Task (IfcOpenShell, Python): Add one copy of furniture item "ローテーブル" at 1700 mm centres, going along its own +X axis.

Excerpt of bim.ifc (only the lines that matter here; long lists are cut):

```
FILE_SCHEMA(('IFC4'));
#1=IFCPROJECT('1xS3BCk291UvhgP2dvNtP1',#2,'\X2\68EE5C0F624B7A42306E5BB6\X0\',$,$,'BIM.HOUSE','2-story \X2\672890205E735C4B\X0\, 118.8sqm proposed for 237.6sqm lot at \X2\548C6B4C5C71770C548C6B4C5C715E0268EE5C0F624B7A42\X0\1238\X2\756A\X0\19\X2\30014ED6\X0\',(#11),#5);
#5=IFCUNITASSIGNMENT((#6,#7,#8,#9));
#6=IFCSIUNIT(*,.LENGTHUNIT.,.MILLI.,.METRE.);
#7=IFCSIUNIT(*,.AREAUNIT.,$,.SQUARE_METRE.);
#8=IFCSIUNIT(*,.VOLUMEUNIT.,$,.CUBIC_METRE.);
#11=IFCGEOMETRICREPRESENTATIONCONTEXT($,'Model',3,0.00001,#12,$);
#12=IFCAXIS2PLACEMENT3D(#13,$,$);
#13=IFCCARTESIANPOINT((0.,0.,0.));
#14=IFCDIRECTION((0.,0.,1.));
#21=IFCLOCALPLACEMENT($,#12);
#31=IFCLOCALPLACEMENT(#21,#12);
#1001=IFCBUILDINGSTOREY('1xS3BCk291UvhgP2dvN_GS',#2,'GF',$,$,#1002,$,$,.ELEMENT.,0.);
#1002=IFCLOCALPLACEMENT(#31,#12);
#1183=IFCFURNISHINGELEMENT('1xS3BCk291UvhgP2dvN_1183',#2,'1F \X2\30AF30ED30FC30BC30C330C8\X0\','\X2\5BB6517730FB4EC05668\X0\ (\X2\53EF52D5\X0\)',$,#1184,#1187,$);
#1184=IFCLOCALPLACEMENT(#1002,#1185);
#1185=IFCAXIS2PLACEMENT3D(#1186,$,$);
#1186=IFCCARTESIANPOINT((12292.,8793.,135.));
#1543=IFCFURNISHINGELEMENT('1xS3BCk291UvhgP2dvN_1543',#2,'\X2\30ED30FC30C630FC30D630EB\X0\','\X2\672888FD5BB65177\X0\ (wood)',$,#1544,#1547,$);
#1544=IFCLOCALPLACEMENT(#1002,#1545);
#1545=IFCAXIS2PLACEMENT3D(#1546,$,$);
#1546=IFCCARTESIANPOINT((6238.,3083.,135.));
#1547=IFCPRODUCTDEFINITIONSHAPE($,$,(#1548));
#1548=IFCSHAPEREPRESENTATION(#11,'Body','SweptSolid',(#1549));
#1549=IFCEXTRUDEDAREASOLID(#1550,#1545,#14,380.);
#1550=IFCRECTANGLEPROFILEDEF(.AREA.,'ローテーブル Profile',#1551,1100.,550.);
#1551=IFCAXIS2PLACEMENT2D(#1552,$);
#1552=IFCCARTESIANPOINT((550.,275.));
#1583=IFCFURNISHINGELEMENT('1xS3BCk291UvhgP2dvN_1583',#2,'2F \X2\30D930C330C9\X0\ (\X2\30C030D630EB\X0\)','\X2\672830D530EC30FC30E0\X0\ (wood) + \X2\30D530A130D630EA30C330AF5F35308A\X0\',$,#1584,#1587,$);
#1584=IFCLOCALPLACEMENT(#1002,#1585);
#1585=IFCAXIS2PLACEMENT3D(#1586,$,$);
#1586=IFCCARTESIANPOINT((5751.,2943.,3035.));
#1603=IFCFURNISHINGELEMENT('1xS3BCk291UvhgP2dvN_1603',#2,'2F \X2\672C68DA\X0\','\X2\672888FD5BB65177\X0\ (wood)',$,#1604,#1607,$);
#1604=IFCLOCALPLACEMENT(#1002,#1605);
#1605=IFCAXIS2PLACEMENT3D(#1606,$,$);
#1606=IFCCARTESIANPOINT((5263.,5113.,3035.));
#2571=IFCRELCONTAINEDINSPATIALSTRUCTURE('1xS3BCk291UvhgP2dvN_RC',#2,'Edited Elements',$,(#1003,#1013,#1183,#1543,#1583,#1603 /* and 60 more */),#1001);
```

```python
import ifcopenshell
import ifcopenshell.api.geometry
import ifcopenshell.api.root
import ifcopenshell.util.element
import ifcopenshell.util.placement
import ifcopenshell.util.unit

model = ifcopenshell.open("bim.ifc")
unit_scale = ifcopenshell.util.unit.calculate_unit_scale(model)


def reuse_history(source, copy):
    """copy_class also copies each property set's owner history, people and application; keep the originals."""
    for rel in copy.IsDefinedBy:
        if rel.is_a("IfcRelDefinesByProperties") and (history := rel.RelatingPropertyDefinition.OwnerHistory):
            rel.RelatingPropertyDefinition.OwnerHistory = source.OwnerHistory
            ifcopenshell.util.element.remove_deep2(model, history)


source = model.by_guid("1xS3BCk291UvhgP2dvN_1543")
base = ifcopenshell.util.placement.get_local_placement(source.ObjectPlacement)
step = base[:3, 0] * 1.7 / unit_scale

for i in range(1, 2):
    copy = ifcopenshell.api.root.copy_class(model, product=source)
    copy.Representation = ifcopenshell.util.element.copy_deep(
        model, source.Representation, exclude=["IfcGeometricRepresentationContext", "IfcRepresentationMap"]
    )
    reuse_history(source, copy)
    matrix = base.copy()
    matrix[:3, 3] += i * step
    print("added at", matrix[:3, 3].round(3) + 0.0)
    ifcopenshell.api.geometry.edit_object_placement(model, product=copy, matrix=matrix, is_si=False)

model.write("bim_rev.ifc")
```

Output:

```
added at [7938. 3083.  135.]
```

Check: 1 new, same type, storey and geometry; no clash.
